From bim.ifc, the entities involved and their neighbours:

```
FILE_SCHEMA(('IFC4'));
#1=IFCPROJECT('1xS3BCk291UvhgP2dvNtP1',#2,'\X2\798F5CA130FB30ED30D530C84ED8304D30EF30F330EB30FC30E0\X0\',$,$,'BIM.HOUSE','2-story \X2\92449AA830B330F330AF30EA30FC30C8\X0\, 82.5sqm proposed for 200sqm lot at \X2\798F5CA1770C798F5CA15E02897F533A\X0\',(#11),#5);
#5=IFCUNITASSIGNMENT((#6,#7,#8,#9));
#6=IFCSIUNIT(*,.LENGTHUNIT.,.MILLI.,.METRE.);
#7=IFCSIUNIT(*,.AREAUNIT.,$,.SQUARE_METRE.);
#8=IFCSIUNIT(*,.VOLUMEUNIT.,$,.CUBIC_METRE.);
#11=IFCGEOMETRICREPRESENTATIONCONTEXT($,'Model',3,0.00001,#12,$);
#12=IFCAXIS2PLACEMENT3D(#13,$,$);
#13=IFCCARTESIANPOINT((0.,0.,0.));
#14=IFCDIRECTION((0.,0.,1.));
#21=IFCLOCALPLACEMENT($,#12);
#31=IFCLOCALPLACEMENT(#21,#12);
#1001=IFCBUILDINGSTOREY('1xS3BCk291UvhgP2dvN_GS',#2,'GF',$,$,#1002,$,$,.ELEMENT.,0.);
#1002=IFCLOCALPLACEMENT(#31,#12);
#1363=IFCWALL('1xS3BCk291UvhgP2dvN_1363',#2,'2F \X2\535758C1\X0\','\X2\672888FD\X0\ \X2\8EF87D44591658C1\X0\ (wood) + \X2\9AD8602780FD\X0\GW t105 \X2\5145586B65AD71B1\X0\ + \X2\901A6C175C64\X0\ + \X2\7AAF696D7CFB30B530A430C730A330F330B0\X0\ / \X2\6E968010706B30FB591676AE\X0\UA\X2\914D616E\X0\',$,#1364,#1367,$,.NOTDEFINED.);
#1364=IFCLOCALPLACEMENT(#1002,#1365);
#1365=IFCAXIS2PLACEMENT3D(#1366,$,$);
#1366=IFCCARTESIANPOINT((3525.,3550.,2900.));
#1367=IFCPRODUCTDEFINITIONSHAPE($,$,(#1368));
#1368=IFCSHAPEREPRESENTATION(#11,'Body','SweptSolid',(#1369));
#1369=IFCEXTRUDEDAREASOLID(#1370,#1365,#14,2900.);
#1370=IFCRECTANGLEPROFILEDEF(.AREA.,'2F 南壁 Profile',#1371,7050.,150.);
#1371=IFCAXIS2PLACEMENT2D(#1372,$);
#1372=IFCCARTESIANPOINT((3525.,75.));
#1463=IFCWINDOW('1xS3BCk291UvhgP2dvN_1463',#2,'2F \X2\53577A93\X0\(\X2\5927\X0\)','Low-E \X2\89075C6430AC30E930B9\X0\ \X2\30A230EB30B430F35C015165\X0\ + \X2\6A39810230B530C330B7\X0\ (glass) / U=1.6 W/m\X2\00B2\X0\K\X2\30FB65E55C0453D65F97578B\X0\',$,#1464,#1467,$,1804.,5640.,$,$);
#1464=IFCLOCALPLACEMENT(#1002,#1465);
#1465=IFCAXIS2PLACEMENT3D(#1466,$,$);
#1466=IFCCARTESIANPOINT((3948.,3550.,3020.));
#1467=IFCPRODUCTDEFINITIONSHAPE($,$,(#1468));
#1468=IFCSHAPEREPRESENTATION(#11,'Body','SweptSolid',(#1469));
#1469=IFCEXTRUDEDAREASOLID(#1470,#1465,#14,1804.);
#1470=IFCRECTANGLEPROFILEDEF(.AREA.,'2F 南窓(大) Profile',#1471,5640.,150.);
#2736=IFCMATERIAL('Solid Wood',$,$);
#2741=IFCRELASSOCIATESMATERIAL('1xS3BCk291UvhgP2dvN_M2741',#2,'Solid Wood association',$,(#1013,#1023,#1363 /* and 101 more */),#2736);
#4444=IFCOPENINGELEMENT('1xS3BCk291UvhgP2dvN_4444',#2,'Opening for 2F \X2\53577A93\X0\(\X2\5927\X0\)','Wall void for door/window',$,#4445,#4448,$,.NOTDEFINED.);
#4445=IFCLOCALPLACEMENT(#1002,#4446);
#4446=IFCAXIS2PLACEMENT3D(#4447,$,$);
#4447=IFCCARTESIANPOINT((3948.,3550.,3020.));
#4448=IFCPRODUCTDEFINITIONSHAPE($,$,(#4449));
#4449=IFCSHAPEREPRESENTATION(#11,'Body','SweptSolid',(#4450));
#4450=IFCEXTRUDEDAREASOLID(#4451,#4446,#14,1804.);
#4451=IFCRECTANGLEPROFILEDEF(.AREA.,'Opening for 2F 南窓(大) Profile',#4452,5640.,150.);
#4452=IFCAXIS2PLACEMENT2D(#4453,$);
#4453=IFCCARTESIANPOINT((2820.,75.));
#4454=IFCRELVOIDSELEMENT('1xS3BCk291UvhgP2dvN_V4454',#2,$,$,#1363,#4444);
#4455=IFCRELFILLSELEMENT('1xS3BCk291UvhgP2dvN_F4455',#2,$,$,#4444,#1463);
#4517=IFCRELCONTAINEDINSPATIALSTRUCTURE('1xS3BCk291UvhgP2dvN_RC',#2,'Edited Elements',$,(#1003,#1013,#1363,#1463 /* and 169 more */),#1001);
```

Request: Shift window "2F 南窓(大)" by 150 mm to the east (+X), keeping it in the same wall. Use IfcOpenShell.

```python
import ifcopenshell
import ifcopenshell.api.geometry
import ifcopenshell.util.placement

model = ifcopenshell.open("bim.ifc")

window = model.by_id(1463)
opening = window.FillsVoids[0].RelatingOpeningElement
wall = opening.VoidsElements[0].RelatingBuildingElement

wall_matrix = ifcopenshell.util.placement.get_local_placement(wall.ObjectPlacement)
shift = wall_matrix[:3, 0] * 150.0
before = ifcopenshell.util.placement.get_local_placement(window.ObjectPlacement)[:3, 3].copy()

# The window is not placed relative to its opening, so move both.
for product in (opening, window):
    matrix = ifcopenshell.util.placement.get_local_placement(product.ObjectPlacement)
    matrix[:3, 3] += shift
    ifcopenshell.api.geometry.edit_object_placement(model, product=product, matrix=matrix, is_si=False)

after = ifcopenshell.util.placement.get_local_placement(window.ObjectPlacement)[:3, 3]
print("window moved by", (after - before).round(3) + 0.0)

model.write("bim_v2.ifc")
```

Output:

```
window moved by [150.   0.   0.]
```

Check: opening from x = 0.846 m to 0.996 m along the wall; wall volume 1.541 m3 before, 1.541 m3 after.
